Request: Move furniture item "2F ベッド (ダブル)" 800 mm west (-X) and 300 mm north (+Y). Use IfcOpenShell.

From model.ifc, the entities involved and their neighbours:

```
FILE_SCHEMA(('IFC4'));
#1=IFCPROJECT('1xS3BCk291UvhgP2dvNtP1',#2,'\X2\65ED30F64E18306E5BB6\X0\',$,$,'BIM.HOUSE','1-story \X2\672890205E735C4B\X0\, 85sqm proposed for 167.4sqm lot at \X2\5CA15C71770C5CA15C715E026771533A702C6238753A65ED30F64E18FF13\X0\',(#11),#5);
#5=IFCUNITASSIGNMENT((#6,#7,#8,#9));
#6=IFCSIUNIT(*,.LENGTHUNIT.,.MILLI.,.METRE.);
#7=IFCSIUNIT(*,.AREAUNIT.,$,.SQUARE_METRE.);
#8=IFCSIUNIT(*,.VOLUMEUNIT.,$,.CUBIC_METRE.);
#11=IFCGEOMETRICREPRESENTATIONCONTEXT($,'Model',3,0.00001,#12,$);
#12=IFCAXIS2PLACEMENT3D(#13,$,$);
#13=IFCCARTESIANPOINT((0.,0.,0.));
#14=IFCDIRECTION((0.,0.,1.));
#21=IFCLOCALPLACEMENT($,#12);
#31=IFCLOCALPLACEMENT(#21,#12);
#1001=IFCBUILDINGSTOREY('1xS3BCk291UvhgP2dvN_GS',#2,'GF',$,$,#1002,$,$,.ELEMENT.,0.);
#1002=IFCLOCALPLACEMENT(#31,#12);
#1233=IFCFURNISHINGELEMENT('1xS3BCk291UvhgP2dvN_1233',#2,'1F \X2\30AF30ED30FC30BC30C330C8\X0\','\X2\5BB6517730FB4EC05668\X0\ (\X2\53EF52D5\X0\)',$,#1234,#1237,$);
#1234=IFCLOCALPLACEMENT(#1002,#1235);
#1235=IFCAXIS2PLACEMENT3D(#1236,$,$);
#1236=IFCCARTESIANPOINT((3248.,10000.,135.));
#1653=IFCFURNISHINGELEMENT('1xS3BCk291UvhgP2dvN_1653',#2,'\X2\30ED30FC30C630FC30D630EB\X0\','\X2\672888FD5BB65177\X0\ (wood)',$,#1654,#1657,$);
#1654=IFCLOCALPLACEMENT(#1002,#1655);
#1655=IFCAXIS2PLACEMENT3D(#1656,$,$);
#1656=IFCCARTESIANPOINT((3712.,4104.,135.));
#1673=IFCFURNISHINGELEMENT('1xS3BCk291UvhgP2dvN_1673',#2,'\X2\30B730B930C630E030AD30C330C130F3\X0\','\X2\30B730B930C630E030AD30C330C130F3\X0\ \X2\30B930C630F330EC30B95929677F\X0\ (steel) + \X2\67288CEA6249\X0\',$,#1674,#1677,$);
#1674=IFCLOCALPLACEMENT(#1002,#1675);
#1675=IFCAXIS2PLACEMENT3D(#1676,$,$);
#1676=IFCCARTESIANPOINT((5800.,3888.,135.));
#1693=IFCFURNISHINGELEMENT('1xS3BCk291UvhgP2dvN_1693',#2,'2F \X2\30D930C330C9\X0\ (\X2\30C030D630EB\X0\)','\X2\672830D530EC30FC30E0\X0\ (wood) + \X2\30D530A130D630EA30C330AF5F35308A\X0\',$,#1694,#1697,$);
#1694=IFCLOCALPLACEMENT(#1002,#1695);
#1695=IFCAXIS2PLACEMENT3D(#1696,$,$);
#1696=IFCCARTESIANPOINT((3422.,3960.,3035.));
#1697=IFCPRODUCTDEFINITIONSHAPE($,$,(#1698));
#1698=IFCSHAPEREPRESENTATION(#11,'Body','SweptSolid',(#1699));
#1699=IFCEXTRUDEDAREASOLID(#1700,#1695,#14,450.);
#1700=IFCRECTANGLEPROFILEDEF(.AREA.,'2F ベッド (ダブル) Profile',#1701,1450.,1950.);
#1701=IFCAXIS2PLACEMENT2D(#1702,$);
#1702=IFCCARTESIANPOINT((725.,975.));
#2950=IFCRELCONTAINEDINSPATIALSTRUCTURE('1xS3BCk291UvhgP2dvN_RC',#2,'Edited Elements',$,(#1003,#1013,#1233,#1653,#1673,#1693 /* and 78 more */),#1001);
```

```python
import ifcopenshell
import ifcopenshell.api.geometry
import ifcopenshell.util.placement
import ifcopenshell.util.unit

model = ifcopenshell.open("model.ifc")
unit_scale = ifcopenshell.util.unit.calculate_unit_scale(model)

item = model.by_guid("1xS3BCk291UvhgP2dvN_1693")
matrix = ifcopenshell.util.placement.get_local_placement(item.ObjectPlacement)
matrix[0, 3] -= 0.8 / unit_scale
matrix[1, 3] += 0.3 / unit_scale
ifcopenshell.api.geometry.edit_object_placement(model, product=item, matrix=matrix, is_si=False)

print(ifcopenshell.util.placement.get_local_placement(item.ObjectPlacement).round(3) + 0.0)

model.write("model_updated.ifc")
```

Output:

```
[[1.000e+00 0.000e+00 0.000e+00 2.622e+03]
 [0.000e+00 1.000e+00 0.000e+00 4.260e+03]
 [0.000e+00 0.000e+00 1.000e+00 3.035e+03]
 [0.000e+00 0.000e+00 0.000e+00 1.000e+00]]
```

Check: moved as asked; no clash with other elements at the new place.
